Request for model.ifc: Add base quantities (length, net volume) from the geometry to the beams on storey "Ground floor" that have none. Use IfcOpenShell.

First a look at what the model holds.

```python
import ifcopenshell
import ifcopenshell.util.element
import ifcopenshell.util.unit

model = ifcopenshell.open("model.ifc")
print(model.schema)
for unit_type in ("LENGTHUNIT", "AREAUNIT", "VOLUMEUNIT"):
    print(unit_type, ifcopenshell.util.unit.calculate_unit_scale(model, unit_type))
storey = next(s for s in model.by_type("IfcBuildingStorey") if s.Name == "Ground floor")
beams = [e for e in ifcopenshell.util.element.get_decomposition(storey) if e.is_a("IfcBeam")]
for e in sorted(beams, key=lambda e: e.id()):
    print(e.id(), e.is_a(), e.Name, list(ifcopenshell.util.element.get_psets(e, qtos_only=True)), sep=" | ")
```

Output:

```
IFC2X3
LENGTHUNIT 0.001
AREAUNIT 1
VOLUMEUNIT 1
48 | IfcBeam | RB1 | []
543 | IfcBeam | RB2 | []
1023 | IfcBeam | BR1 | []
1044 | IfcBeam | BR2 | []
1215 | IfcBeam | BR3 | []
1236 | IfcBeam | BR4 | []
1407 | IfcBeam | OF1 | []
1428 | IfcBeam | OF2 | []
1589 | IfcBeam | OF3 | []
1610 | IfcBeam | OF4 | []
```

```python
import ifcopenshell
import ifcopenshell.api.pset
import ifcopenshell.geom
import ifcopenshell.util.element
import ifcopenshell.util.shape
import ifcopenshell.util.unit

model = ifcopenshell.open("model.ifc")
unit_scale = ifcopenshell.util.unit.calculate_unit_scale(model)
volume_scale = ifcopenshell.util.unit.calculate_unit_scale(model, "VOLUMEUNIT")
settings = ifcopenshell.geom.settings()

storey = next(s for s in model.by_type("IfcBuildingStorey") if s.Name == "Ground floor")
beams = [e for e in ifcopenshell.util.element.get_decomposition(storey) if e.is_a("IfcBeam")]

for e in sorted(beams, key=lambda e: e.id()):
    if ifcopenshell.util.element.get_psets(e, qtos_only=True, should_inherit=False):
        continue
    # Geometry comes back in metres, in the element's own axes.
    shape = ifcopenshell.geom.create_shape(settings, e)
    values = {
        "Length": ifcopenshell.util.shape.get_max_xyz(shape.geometry) / unit_scale,
        "NetVolume": ifcopenshell.util.shape.get_volume(shape.geometry) / volume_scale,
    }
    qto = ifcopenshell.api.pset.add_qto(model, product=e, name="BaseQuantities")
    ifcopenshell.api.pset.edit_qto(model, qto=qto, properties=values)
    print(e.id(), {k: round(v, 3) for k, v in values.items()})

model.write("model_updated.ifc")
```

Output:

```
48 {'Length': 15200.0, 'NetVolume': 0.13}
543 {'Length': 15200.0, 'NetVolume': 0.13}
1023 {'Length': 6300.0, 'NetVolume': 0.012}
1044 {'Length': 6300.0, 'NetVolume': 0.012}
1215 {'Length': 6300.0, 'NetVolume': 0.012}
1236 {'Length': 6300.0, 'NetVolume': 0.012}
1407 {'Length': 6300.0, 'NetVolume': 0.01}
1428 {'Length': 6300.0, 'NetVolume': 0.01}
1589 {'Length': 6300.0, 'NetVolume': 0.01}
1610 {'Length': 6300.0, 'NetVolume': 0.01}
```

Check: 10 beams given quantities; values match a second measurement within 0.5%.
